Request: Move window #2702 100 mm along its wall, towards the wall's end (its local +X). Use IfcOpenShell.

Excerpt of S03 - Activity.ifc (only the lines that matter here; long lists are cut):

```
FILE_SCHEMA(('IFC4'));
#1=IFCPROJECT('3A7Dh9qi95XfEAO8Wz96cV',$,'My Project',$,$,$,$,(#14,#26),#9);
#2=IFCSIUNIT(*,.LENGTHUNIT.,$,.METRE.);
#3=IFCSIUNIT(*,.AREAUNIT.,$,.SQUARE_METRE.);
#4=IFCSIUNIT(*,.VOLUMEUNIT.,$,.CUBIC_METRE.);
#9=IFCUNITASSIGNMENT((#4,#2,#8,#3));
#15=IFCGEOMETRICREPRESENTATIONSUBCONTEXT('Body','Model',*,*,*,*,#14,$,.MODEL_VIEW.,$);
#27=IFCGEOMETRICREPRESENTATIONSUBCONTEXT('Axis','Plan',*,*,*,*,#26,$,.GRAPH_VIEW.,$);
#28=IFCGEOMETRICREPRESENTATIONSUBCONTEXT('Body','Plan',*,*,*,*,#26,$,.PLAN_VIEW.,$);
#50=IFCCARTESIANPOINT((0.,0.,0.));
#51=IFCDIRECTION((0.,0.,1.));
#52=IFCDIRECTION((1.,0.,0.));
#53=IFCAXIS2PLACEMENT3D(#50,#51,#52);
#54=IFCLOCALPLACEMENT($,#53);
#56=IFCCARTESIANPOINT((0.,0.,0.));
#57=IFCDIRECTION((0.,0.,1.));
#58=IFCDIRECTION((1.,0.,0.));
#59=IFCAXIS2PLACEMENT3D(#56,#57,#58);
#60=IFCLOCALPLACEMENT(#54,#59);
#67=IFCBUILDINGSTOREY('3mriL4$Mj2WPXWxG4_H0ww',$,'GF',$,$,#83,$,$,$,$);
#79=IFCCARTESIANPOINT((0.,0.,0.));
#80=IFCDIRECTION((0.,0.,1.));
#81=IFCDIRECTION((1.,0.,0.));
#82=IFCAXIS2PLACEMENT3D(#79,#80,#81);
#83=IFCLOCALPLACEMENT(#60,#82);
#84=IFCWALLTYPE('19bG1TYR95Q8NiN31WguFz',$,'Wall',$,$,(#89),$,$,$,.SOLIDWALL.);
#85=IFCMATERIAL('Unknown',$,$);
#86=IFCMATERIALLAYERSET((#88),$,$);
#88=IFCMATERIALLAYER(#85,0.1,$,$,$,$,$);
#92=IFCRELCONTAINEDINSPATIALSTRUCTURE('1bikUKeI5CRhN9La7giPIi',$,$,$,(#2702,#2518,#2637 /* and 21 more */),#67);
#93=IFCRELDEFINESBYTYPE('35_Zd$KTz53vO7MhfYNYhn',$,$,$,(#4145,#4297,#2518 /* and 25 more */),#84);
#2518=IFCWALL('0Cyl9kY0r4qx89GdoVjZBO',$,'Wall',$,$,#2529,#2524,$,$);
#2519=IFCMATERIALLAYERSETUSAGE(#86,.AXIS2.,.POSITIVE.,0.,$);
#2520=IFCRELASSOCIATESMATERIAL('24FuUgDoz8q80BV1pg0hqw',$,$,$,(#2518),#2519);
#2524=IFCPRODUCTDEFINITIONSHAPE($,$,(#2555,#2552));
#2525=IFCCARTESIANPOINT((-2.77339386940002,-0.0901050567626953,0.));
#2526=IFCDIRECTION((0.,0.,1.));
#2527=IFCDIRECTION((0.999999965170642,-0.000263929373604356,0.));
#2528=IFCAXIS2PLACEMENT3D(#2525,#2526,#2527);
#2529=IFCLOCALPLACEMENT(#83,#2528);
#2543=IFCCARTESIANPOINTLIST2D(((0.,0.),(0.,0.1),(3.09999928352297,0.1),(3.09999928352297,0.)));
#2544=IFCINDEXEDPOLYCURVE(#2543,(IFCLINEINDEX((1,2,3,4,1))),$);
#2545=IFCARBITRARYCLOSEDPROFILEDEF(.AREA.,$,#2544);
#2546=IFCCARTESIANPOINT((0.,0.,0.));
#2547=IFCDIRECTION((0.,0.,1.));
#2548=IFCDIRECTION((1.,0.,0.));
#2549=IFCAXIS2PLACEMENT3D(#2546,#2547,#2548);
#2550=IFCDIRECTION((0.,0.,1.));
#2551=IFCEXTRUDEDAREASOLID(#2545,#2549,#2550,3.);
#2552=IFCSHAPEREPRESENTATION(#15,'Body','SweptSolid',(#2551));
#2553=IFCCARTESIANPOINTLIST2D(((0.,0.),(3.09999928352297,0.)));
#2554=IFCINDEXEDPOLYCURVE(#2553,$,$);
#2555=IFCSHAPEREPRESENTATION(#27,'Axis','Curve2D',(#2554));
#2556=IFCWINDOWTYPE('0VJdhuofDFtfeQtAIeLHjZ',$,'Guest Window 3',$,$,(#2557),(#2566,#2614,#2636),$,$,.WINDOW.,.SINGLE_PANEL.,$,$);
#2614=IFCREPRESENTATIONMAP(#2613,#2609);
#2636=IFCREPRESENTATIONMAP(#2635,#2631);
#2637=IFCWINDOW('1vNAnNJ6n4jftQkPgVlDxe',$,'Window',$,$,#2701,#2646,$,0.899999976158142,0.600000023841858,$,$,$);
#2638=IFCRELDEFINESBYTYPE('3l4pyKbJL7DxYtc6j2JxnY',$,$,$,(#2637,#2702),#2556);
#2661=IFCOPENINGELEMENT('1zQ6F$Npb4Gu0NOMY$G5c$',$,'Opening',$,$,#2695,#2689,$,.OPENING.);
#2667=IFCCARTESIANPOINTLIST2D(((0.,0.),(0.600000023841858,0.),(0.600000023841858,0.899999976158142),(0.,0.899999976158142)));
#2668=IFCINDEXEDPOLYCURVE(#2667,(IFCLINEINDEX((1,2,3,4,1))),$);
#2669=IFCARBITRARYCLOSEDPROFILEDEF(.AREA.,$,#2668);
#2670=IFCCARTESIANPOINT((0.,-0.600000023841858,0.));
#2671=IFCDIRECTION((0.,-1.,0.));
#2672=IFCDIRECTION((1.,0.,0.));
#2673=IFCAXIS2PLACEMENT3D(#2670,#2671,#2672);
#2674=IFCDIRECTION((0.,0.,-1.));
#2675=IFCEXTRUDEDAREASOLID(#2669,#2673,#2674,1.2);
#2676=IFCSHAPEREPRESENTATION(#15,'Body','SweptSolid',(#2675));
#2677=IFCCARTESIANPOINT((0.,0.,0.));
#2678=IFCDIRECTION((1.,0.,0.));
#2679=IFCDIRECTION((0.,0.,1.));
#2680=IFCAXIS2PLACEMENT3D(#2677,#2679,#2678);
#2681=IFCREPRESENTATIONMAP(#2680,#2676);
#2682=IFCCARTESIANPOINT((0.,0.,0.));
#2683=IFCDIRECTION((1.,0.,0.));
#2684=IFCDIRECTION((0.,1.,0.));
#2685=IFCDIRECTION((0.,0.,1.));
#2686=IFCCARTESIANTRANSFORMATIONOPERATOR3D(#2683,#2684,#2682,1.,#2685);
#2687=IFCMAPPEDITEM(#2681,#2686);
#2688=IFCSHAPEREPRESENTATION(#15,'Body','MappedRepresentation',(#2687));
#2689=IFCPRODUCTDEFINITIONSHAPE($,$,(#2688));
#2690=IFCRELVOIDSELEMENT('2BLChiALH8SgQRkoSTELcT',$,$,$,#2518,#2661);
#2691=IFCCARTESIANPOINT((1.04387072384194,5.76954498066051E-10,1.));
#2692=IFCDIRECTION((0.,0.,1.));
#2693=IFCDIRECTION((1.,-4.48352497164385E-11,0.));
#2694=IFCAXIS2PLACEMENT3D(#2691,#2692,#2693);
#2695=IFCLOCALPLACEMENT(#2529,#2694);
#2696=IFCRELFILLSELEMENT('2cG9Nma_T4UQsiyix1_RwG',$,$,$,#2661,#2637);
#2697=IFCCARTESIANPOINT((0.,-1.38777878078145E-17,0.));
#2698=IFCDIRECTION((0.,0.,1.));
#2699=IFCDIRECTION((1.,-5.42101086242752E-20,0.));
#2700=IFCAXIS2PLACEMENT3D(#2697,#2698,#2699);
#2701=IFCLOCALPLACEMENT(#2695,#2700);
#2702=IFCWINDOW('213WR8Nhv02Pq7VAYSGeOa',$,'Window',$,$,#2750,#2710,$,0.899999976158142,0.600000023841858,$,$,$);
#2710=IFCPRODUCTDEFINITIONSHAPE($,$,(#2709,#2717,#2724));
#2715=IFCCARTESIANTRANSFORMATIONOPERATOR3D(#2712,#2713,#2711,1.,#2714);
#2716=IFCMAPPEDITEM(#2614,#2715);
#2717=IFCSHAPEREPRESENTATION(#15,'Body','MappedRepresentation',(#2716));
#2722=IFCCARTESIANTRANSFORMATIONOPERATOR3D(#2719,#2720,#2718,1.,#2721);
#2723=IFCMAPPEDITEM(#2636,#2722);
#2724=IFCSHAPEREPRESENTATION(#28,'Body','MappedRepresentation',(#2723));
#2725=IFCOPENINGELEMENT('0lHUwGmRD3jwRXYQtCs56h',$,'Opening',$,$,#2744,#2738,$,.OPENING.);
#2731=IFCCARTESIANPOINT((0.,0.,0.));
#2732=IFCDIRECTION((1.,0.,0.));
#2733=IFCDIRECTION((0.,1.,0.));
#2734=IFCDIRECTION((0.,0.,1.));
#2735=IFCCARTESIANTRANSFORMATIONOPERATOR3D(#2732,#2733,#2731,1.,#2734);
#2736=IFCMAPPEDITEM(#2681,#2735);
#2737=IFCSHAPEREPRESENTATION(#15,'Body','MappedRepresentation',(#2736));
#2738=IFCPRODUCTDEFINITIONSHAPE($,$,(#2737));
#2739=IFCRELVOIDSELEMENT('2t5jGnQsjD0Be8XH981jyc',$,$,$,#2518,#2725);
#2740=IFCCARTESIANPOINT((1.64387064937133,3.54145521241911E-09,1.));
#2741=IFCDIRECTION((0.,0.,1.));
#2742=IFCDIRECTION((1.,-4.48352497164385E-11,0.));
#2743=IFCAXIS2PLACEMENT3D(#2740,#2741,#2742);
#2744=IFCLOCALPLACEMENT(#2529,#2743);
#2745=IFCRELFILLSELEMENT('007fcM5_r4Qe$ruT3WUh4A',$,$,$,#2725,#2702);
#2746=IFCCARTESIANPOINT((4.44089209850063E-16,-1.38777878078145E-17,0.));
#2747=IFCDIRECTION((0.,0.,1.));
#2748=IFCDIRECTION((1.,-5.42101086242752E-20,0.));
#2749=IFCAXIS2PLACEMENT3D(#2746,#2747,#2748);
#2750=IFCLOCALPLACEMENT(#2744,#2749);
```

```python
import ifcopenshell
import ifcopenshell.api.geometry
import ifcopenshell.util.placement
import ifcopenshell.util.unit

model = ifcopenshell.open("S03 - Activity.ifc")
unit_scale = ifcopenshell.util.unit.calculate_unit_scale(model)

window = model.by_guid("213WR8Nhv02Pq7VAYSGeOa")
opening = window.FillsVoids[0].RelatingOpeningElement
wall = opening.VoidsElements[0].RelatingBuildingElement

wall_matrix = ifcopenshell.util.placement.get_local_placement(wall.ObjectPlacement)
shift = wall_matrix[:3, 0] * 0.1 / unit_scale
before = ifcopenshell.util.placement.get_local_placement(window.ObjectPlacement)[:3, 3].copy()

# The window is placed relative to its opening, so it follows when the opening moves.
matrix = ifcopenshell.util.placement.get_local_placement(opening.ObjectPlacement)
matrix[:3, 3] += shift
ifcopenshell.api.geometry.edit_object_placement(
    model, product=opening, matrix=matrix, is_si=False, should_transform_children=True
)

after = ifcopenshell.util.placement.get_local_placement(window.ObjectPlacement)[:3, 3]
print("window moved by", (after - before).round(3) + 0.0)

model.write("S03 - Activity_rev.ifc")
```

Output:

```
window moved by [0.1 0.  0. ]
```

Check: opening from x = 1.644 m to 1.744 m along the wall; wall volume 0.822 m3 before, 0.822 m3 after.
